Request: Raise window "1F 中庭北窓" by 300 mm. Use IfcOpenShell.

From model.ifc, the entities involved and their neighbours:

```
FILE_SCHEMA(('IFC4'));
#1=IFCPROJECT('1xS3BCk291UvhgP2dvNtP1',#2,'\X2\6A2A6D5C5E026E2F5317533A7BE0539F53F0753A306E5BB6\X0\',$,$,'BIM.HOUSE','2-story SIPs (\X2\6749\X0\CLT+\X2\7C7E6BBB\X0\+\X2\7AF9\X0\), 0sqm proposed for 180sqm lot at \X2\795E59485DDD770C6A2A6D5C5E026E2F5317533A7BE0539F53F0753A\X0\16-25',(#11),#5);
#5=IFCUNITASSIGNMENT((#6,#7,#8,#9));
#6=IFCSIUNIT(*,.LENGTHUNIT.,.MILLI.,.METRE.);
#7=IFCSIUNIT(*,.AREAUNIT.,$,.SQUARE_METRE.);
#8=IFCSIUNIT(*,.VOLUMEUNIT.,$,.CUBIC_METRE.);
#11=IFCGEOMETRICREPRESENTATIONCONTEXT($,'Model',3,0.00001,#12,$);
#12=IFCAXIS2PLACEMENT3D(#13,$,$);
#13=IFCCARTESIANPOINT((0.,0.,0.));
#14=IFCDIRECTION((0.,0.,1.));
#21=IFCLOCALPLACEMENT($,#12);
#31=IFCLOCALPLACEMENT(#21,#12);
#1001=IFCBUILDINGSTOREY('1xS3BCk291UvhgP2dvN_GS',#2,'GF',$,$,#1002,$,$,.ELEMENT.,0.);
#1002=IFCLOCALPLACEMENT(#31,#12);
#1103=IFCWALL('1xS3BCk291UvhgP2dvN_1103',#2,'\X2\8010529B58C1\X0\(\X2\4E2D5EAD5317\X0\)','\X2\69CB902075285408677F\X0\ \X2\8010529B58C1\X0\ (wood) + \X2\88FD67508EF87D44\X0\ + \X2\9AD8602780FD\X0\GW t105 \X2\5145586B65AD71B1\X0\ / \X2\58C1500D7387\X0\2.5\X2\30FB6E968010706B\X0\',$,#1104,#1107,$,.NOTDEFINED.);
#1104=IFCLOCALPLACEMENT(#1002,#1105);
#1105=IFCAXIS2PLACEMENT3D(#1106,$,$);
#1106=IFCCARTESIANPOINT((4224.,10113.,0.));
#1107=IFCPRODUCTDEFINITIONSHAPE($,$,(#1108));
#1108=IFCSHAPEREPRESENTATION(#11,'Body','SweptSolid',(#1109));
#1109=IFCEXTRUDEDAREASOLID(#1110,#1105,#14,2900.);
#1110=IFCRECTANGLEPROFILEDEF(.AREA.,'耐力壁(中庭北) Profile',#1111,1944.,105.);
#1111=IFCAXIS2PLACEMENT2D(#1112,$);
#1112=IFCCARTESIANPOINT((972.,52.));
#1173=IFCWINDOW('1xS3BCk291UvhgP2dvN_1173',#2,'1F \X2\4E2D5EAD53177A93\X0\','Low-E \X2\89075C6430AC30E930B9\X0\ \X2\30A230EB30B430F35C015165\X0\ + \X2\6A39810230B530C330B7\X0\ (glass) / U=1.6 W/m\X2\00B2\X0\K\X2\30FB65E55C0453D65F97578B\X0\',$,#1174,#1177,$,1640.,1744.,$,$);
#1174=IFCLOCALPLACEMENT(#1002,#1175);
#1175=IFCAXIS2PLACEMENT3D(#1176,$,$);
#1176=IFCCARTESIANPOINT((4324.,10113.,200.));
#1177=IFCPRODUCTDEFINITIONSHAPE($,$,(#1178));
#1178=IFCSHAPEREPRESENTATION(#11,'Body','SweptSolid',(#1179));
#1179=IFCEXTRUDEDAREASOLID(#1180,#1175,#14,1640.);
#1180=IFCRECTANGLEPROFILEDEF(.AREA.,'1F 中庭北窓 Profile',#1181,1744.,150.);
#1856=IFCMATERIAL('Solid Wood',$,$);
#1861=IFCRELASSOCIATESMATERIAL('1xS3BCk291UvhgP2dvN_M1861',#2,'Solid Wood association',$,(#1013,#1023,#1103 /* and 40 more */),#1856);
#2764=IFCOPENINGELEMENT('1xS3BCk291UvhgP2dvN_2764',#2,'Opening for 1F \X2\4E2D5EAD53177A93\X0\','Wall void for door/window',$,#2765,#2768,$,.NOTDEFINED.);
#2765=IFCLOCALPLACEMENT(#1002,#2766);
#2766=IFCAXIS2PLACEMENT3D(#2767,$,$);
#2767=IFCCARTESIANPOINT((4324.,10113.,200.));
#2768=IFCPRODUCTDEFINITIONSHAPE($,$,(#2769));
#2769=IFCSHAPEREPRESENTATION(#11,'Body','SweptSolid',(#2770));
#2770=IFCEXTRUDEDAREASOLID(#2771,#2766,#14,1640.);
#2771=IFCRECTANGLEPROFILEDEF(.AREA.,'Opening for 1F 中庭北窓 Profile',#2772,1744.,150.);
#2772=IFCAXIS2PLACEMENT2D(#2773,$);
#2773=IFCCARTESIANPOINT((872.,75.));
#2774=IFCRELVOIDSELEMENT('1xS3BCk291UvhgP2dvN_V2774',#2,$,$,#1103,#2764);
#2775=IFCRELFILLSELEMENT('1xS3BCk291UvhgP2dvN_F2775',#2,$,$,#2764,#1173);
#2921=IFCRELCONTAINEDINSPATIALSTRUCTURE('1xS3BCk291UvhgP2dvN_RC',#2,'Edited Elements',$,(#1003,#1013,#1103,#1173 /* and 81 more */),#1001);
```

```python
import numpy as np
import ifcopenshell
import ifcopenshell.api.geometry
import ifcopenshell.util.placement
import ifcopenshell.util.unit

model = ifcopenshell.open("model.ifc")
unit_scale = ifcopenshell.util.unit.calculate_unit_scale(model)

window = model.by_guid("1xS3BCk291UvhgP2dvN_1173")
opening = window.FillsVoids[0].RelatingOpeningElement
dz = 0.3 / unit_scale

shift = np.array([0.0, 0.0, dz])
# The window is not placed relative to its opening, so move both.
for product in (opening, window):
    matrix = ifcopenshell.util.placement.get_local_placement(product.ObjectPlacement)
    matrix[:3, 3] += shift
    ifcopenshell.api.geometry.edit_object_placement(model, product=product, matrix=matrix, is_si=False)

print(f"moved by {dz * unit_scale:+.3f} m")

model.write("model_edited.ifc")
```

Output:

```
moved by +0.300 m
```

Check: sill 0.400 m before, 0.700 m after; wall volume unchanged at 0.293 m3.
